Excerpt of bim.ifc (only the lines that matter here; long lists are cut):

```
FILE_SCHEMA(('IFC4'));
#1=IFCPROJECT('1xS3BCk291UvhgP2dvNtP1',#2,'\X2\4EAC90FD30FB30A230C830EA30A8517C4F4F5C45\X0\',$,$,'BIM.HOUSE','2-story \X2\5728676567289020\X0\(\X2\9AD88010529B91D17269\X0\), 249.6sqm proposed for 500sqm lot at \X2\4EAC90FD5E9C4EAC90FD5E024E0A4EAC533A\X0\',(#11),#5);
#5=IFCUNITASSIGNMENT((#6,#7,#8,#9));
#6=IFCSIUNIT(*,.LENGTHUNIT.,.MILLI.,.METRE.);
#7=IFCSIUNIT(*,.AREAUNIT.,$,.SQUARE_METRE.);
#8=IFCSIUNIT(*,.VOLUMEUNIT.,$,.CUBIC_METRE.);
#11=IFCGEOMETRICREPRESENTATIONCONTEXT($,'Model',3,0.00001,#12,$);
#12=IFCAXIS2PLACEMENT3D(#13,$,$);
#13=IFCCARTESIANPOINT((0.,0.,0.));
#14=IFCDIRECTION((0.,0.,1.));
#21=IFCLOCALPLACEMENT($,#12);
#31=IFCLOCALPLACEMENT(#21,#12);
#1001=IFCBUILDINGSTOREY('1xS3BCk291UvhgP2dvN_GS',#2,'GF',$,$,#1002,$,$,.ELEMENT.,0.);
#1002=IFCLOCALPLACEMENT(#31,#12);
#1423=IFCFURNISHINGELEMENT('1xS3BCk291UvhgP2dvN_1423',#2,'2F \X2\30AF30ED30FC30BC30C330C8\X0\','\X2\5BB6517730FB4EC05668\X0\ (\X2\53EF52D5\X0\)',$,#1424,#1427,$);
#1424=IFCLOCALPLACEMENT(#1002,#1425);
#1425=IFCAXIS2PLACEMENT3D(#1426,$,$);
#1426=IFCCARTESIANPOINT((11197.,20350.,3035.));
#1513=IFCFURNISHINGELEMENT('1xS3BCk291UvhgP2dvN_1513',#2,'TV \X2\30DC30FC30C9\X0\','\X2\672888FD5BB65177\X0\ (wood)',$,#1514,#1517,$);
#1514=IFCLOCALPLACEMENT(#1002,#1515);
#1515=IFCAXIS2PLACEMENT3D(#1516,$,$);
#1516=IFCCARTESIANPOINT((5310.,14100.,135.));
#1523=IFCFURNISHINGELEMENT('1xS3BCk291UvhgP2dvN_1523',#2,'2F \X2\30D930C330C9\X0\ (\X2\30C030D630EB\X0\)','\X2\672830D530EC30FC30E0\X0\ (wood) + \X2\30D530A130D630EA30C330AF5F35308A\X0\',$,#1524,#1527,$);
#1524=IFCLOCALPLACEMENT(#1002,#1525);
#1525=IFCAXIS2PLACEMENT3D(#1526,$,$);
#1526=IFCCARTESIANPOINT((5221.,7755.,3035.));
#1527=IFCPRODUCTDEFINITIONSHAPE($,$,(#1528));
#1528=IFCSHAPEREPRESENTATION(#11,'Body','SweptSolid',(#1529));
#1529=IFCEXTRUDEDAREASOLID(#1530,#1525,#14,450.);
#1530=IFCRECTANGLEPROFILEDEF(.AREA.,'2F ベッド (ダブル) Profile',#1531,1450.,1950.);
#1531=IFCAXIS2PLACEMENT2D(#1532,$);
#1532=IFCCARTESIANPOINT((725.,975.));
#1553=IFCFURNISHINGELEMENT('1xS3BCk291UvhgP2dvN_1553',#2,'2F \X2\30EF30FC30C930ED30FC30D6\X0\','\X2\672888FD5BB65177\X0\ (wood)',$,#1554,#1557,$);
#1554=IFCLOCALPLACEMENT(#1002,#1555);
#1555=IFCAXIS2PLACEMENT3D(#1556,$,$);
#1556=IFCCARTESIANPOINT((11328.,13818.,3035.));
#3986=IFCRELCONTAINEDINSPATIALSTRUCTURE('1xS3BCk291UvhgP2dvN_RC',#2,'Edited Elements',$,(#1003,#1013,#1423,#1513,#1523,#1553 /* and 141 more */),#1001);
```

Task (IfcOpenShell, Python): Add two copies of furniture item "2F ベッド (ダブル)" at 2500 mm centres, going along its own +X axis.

```python
import ifcopenshell
import ifcopenshell.api.geometry
import ifcopenshell.api.root
import ifcopenshell.util.element
import ifcopenshell.util.placement

model = ifcopenshell.open("bim.ifc")


def reuse_history(source, copy):
    """copy_class also copies each property set's owner history, people and application; keep the originals."""
    for rel in copy.IsDefinedBy:
        if rel.is_a("IfcRelDefinesByProperties") and (history := rel.RelatingPropertyDefinition.OwnerHistory):
            rel.RelatingPropertyDefinition.OwnerHistory = source.OwnerHistory
            ifcopenshell.util.element.remove_deep2(model, history)


source = model.by_guid("1xS3BCk291UvhgP2dvN_1523")
base = ifcopenshell.util.placement.get_local_placement(source.ObjectPlacement)
step = base[:3, 0] * 2500.0

for i in range(1, 3):
    copy = ifcopenshell.api.root.copy_class(model, product=source)
    copy.Representation = ifcopenshell.util.element.copy_deep(
        model, source.Representation, exclude=["IfcGeometricRepresentationContext", "IfcRepresentationMap"]
    )
    reuse_history(source, copy)
    matrix = base.copy()
    matrix[:3, 3] += i * step
    print("added at", matrix[:3, 3].round(3) + 0.0)
    ifcopenshell.api.geometry.edit_object_placement(model, product=copy, matrix=matrix, is_si=False)

model.write("bim_edited.ifc")
```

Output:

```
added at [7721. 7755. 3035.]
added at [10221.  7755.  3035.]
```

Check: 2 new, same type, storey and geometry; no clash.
